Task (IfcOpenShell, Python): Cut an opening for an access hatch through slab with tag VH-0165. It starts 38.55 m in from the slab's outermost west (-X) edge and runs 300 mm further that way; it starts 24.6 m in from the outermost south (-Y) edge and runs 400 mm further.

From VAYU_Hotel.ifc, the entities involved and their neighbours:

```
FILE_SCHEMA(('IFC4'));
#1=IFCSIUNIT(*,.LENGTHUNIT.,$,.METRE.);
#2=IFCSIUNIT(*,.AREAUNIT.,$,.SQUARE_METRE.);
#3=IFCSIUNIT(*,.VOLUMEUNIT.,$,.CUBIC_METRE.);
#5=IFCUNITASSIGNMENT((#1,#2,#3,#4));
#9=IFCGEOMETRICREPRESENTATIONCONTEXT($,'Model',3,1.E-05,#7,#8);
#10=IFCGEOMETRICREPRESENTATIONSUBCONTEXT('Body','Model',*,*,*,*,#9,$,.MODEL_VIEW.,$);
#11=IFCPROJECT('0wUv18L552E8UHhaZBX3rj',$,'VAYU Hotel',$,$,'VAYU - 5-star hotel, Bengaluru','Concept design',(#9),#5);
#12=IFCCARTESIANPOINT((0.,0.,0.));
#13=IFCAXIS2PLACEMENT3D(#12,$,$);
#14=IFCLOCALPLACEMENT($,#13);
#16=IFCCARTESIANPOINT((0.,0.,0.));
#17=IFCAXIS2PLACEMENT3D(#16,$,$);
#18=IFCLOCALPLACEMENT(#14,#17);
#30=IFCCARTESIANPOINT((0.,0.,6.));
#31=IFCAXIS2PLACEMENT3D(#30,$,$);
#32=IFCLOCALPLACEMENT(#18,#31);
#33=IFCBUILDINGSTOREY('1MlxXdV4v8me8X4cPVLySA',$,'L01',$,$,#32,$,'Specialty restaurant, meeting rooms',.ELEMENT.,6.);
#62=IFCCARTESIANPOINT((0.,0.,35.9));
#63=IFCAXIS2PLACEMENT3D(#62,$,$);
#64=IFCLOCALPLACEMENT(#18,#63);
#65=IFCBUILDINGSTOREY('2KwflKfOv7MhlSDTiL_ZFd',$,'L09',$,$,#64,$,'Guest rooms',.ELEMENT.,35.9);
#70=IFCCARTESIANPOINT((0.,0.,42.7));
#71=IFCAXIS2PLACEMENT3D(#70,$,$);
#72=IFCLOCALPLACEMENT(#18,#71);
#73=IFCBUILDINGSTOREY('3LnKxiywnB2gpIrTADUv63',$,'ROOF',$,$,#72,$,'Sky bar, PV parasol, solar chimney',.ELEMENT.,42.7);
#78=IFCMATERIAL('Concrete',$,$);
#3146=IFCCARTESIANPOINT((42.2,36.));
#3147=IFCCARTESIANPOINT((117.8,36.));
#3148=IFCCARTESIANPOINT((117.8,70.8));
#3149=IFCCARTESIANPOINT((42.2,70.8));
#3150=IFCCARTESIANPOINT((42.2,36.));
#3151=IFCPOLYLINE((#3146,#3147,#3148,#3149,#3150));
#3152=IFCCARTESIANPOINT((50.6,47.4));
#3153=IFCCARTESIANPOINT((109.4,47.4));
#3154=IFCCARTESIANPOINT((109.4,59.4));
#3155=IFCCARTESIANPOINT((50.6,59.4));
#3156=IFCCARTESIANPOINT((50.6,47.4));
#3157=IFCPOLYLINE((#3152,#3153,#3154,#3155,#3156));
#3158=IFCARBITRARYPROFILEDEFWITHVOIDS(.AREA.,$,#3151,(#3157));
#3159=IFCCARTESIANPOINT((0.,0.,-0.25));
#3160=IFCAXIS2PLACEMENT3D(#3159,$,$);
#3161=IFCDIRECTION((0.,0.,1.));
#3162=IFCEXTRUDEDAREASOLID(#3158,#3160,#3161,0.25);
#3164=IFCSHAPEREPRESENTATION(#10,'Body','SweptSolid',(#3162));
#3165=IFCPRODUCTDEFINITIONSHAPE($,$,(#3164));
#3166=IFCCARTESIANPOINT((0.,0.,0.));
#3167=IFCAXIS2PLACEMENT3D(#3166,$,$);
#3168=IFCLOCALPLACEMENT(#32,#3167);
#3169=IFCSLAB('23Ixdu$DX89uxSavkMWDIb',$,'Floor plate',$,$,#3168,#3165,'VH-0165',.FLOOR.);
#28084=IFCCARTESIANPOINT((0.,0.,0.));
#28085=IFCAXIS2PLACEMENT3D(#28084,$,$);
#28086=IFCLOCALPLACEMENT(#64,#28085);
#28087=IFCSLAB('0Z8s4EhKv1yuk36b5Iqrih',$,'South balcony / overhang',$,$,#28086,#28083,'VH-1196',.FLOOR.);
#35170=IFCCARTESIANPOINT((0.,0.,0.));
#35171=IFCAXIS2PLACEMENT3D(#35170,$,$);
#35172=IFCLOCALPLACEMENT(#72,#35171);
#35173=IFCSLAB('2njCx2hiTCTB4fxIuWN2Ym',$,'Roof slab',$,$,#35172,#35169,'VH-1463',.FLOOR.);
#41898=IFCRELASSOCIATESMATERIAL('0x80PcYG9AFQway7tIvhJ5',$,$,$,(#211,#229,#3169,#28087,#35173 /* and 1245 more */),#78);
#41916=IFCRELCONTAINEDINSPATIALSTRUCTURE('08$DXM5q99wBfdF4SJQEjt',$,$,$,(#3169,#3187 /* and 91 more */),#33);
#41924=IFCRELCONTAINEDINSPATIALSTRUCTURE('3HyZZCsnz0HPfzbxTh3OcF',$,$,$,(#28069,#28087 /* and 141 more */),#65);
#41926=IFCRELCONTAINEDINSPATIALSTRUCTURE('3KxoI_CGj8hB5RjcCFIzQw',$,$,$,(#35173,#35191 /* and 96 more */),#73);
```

```python
import numpy as np
import ifcopenshell
import ifcopenshell.api.feature
import ifcopenshell.api.geometry
import ifcopenshell.api.root
import ifcopenshell.geom
import ifcopenshell.util.placement
import ifcopenshell.util.representation
import ifcopenshell.util.shape
import ifcopenshell.util.unit

model = ifcopenshell.open("VAYU_Hotel.ifc")
unit_scale = ifcopenshell.util.unit.calculate_unit_scale(model)
settings = ifcopenshell.geom.settings()


def volume(element):
    """Net volume in cubic metres, openings subtracted."""
    shape = ifcopenshell.geom.create_shape(settings, element)
    return ifcopenshell.util.shape.get_volume(shape.geometry)


slab = model.by_guid("23Ixdu$DX89uxSavkMWDIb")
before = volume(slab)

# Extent in the slab's own axes, in metres. The edges named are its -X and -Y sides.
slab_shape = ifcopenshell.geom.create_shape(settings, slab)
vertices = ifcopenshell.util.shape.get_vertices(slab_shape.geometry)
x_min, y_min, bottom = vertices.min(axis=0)
top = vertices[:, 2].max()

opening = ifcopenshell.api.root.create_entity(model, ifc_class="IfcOpeningElement", name="Access hatch opening", predefined_type="OPENING")
context = ifcopenshell.util.representation.get_context(model, "Model", "Body", "MODEL_VIEW")
width, depth = 0.3, 0.4
outline = [(0.0, 0.0), (width, 0.0), (width, depth), (0.0, depth), (0.0, 0.0)]
# Overshoot both faces by 50 mm so the cut is clean.
shape = ifcopenshell.api.geometry.add_slab_representation(
    model, context=context, depth=top - bottom + 0.1, polyline=outline
)
ifcopenshell.api.geometry.assign_representation(model, product=opening, representation=shape)

matrix = ifcopenshell.util.placement.get_local_placement(slab.ObjectPlacement)
matrix[:, 3] = matrix @ np.append(np.array([x_min + 38.55, y_min + 24.6, bottom - 0.05]) / unit_scale, 1.0)
ifcopenshell.api.geometry.edit_object_placement(model, product=opening, matrix=matrix, is_si=False)
ifcopenshell.api.feature.add_feature(model, feature=opening, element=slab)

after = volume(slab)

print(f"slab volume {before:.3f} -> {after:.3f} m3")

model.write("VAYU_Hotel_updated.ifc")
```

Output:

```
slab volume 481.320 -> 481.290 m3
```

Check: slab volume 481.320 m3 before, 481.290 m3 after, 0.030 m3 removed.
